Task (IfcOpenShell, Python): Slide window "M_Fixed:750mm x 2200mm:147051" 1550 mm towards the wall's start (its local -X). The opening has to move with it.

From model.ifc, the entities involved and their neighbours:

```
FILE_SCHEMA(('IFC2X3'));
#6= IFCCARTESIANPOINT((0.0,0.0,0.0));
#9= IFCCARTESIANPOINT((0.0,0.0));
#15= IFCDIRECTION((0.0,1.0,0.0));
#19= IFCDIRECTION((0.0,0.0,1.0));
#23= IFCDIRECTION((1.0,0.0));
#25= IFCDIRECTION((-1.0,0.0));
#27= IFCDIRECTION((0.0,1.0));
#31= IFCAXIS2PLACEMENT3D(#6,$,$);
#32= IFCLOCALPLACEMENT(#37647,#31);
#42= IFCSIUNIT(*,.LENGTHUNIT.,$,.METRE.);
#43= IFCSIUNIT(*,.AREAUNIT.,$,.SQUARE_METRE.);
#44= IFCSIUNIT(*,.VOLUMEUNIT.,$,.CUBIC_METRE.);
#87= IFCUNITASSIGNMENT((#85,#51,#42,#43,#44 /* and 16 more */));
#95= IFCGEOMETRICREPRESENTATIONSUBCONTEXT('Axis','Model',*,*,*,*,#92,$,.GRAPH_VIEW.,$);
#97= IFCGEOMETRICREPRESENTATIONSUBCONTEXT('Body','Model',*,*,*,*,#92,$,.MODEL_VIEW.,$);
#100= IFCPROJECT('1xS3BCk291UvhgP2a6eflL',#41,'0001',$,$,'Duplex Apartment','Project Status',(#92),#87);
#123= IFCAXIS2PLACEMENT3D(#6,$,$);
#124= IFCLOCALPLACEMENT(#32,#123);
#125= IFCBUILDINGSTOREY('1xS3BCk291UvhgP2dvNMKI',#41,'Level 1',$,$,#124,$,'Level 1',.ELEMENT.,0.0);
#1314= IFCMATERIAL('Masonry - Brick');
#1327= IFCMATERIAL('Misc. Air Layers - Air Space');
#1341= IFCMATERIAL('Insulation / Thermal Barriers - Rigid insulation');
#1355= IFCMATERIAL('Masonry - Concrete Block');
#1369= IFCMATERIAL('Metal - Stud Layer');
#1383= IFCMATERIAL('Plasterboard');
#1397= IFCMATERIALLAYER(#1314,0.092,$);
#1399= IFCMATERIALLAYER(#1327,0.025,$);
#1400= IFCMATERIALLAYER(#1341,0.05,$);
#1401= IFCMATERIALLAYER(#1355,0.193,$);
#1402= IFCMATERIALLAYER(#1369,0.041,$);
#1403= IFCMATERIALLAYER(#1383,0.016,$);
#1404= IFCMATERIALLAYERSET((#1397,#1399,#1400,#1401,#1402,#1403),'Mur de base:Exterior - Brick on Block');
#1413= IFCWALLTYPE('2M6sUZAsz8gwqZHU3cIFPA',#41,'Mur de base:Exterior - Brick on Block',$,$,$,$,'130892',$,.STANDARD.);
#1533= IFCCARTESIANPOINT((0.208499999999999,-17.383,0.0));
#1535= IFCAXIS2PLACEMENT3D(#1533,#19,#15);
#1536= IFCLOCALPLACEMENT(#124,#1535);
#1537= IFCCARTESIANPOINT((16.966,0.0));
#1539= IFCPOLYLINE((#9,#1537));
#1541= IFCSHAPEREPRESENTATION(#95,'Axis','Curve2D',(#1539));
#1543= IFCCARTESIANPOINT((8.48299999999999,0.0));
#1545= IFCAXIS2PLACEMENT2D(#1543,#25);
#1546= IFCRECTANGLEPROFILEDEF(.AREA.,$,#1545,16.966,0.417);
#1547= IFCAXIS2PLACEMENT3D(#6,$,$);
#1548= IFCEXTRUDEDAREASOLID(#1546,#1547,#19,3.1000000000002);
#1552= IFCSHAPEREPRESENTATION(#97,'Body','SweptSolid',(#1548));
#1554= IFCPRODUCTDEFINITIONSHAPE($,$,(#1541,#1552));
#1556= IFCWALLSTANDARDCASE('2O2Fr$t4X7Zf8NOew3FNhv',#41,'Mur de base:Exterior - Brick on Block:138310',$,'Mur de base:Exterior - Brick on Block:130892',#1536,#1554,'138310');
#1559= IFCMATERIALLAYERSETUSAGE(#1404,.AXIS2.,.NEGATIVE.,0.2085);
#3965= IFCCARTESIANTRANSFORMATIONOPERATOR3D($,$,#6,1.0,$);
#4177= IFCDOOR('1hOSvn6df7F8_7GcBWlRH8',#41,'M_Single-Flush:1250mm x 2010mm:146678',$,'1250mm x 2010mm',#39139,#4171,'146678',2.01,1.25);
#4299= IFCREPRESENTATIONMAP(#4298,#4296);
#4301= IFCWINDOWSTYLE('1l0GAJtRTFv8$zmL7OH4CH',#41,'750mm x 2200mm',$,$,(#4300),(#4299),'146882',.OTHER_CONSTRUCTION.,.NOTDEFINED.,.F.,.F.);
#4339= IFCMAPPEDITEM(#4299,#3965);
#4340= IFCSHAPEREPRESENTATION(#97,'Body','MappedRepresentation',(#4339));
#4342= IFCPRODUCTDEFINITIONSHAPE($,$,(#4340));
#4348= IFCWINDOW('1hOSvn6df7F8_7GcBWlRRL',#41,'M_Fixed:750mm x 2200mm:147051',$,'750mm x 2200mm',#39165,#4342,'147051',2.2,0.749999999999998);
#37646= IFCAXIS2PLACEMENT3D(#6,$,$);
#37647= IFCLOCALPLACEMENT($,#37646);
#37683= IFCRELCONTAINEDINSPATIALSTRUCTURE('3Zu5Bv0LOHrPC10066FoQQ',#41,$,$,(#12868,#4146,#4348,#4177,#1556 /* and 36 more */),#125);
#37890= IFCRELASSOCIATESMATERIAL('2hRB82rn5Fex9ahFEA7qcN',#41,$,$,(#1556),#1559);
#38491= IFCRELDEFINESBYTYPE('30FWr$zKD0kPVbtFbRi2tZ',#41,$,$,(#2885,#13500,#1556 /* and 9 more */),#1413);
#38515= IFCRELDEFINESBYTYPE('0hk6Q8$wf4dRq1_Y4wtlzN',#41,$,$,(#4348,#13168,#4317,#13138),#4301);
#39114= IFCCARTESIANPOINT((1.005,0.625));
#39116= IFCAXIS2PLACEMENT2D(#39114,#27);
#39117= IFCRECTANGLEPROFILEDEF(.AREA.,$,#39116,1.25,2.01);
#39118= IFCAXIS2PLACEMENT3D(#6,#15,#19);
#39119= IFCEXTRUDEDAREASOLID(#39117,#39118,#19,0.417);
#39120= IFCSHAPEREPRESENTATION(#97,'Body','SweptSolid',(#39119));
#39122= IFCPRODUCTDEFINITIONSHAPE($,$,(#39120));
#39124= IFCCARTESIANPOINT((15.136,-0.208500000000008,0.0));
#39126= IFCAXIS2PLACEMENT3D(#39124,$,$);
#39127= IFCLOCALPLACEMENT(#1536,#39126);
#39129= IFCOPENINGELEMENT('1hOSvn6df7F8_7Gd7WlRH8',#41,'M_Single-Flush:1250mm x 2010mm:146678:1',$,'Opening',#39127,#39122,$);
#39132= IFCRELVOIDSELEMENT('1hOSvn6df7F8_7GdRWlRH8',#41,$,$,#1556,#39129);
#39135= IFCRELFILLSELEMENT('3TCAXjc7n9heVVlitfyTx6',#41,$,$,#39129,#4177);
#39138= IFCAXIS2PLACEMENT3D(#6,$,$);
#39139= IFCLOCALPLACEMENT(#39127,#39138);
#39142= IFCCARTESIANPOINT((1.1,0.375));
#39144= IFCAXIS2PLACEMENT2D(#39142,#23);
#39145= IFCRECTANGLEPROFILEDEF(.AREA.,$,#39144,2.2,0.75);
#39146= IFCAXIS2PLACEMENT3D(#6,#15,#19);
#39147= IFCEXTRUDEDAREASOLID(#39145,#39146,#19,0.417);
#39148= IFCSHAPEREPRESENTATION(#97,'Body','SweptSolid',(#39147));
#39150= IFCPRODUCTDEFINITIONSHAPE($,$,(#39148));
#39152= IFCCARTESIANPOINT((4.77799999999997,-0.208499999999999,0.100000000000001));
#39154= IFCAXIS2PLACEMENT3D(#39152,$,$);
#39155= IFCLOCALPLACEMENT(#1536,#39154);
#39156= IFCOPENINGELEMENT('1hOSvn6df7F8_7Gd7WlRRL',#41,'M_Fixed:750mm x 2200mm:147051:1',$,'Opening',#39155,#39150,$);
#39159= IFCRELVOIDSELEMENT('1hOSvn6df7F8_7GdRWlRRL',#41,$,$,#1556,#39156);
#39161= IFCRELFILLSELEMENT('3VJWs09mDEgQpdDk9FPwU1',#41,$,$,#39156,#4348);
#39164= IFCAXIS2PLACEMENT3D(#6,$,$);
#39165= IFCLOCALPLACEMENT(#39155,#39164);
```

```python
import ifcopenshell
import ifcopenshell.api.geometry
import ifcopenshell.util.placement
import ifcopenshell.util.unit

model = ifcopenshell.open("model.ifc")
unit_scale = ifcopenshell.util.unit.calculate_unit_scale(model)

window = model.by_guid("1hOSvn6df7F8_7GcBWlRRL")
opening = window.FillsVoids[0].RelatingOpeningElement
wall = opening.VoidsElements[0].RelatingBuildingElement

wall_matrix = ifcopenshell.util.placement.get_local_placement(wall.ObjectPlacement)
shift = wall_matrix[:3, 0] * -1.55 / unit_scale
before = ifcopenshell.util.placement.get_local_placement(window.ObjectPlacement)[:3, 3].copy()

# The window is placed relative to its opening, so it follows when the opening moves.
matrix = ifcopenshell.util.placement.get_local_placement(opening.ObjectPlacement)
matrix[:3, 3] += shift
ifcopenshell.api.geometry.edit_object_placement(
    model, product=opening, matrix=matrix, is_si=False, should_transform_children=True
)

after = ifcopenshell.util.placement.get_local_placement(window.ObjectPlacement)[:3, 3]
print("window moved by", (after - before).round(3) + 0.0)

model.write("model_rev.ifc")
```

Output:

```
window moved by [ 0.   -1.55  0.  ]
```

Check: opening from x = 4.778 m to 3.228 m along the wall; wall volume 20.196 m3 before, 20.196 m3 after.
